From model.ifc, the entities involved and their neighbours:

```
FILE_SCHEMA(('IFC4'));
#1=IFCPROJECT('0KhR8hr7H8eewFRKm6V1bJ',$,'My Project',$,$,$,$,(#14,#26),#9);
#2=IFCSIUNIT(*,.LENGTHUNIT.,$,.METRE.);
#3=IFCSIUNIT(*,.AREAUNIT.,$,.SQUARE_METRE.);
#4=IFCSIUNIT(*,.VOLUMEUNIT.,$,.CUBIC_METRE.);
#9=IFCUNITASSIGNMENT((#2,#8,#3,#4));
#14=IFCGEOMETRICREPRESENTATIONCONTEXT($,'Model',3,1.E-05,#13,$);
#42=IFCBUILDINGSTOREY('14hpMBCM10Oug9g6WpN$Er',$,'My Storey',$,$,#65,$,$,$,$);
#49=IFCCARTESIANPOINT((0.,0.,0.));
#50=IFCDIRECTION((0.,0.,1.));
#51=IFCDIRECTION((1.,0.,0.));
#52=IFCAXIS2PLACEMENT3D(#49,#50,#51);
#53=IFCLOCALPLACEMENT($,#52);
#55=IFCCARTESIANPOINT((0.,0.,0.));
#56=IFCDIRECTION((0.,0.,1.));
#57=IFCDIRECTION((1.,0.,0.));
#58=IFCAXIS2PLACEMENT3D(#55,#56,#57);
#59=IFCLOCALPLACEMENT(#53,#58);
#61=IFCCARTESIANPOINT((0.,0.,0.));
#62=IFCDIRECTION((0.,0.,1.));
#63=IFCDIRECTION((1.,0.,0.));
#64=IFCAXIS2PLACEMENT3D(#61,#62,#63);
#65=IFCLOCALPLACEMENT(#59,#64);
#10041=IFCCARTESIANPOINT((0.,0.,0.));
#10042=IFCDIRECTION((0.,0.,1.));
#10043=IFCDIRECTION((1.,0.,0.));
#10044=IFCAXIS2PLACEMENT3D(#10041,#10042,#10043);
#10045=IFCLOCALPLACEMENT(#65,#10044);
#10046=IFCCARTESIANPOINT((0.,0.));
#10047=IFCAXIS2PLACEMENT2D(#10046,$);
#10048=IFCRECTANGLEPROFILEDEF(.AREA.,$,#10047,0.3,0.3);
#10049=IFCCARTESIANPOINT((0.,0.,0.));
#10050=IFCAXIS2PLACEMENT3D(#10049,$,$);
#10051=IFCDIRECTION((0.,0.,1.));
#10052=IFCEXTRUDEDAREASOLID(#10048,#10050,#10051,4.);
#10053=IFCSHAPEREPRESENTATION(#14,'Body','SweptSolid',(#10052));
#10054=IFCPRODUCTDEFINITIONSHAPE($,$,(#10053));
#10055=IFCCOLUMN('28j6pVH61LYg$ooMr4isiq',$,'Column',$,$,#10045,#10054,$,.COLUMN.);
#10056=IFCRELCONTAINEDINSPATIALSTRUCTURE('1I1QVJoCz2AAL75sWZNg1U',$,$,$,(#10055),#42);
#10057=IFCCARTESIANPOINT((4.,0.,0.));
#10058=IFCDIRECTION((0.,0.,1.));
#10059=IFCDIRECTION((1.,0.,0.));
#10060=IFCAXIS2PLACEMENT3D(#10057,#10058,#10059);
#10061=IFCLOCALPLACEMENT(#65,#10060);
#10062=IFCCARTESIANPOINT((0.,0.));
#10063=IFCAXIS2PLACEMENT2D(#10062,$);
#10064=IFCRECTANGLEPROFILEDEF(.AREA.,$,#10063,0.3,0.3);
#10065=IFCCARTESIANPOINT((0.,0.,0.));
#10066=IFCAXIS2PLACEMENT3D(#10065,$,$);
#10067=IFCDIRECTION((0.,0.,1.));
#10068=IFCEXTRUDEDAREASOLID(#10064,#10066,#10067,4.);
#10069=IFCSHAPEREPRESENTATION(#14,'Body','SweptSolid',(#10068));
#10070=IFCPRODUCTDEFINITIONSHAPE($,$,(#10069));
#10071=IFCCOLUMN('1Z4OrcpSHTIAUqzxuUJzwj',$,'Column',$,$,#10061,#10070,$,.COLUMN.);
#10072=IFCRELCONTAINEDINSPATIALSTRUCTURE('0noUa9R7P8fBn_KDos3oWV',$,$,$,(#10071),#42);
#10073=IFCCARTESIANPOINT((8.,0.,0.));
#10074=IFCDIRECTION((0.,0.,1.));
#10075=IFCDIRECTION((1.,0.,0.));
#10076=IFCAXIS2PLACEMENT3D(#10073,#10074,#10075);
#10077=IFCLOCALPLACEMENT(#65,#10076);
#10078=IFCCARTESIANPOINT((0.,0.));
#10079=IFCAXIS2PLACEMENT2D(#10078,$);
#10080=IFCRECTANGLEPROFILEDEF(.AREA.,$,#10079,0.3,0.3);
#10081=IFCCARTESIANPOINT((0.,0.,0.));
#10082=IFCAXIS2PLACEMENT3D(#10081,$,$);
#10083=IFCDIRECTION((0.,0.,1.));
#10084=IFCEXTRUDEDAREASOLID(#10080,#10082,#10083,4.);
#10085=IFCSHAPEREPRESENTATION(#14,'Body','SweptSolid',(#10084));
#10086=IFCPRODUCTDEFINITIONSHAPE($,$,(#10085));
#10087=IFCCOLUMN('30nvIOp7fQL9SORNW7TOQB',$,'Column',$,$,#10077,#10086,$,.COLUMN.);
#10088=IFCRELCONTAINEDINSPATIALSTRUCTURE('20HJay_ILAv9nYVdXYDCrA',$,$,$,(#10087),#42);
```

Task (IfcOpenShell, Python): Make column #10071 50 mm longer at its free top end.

```python
import ifcopenshell

model = ifcopenshell.open("model.ifc")

member = model.by_id(10071)
change = 0.05

# The extrusion runs towards the end named, so only its depth changes.
body = next(r for r in member.Representation.Representations if r.RepresentationIdentifier == "Body")
solid = body.Items[0]
old_length = solid.Depth
solid.Depth += change

print(f"length {old_length:g} -> {solid.Depth:g}")

model.write("model-out.ifc")
```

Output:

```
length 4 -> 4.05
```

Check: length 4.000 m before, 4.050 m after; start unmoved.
